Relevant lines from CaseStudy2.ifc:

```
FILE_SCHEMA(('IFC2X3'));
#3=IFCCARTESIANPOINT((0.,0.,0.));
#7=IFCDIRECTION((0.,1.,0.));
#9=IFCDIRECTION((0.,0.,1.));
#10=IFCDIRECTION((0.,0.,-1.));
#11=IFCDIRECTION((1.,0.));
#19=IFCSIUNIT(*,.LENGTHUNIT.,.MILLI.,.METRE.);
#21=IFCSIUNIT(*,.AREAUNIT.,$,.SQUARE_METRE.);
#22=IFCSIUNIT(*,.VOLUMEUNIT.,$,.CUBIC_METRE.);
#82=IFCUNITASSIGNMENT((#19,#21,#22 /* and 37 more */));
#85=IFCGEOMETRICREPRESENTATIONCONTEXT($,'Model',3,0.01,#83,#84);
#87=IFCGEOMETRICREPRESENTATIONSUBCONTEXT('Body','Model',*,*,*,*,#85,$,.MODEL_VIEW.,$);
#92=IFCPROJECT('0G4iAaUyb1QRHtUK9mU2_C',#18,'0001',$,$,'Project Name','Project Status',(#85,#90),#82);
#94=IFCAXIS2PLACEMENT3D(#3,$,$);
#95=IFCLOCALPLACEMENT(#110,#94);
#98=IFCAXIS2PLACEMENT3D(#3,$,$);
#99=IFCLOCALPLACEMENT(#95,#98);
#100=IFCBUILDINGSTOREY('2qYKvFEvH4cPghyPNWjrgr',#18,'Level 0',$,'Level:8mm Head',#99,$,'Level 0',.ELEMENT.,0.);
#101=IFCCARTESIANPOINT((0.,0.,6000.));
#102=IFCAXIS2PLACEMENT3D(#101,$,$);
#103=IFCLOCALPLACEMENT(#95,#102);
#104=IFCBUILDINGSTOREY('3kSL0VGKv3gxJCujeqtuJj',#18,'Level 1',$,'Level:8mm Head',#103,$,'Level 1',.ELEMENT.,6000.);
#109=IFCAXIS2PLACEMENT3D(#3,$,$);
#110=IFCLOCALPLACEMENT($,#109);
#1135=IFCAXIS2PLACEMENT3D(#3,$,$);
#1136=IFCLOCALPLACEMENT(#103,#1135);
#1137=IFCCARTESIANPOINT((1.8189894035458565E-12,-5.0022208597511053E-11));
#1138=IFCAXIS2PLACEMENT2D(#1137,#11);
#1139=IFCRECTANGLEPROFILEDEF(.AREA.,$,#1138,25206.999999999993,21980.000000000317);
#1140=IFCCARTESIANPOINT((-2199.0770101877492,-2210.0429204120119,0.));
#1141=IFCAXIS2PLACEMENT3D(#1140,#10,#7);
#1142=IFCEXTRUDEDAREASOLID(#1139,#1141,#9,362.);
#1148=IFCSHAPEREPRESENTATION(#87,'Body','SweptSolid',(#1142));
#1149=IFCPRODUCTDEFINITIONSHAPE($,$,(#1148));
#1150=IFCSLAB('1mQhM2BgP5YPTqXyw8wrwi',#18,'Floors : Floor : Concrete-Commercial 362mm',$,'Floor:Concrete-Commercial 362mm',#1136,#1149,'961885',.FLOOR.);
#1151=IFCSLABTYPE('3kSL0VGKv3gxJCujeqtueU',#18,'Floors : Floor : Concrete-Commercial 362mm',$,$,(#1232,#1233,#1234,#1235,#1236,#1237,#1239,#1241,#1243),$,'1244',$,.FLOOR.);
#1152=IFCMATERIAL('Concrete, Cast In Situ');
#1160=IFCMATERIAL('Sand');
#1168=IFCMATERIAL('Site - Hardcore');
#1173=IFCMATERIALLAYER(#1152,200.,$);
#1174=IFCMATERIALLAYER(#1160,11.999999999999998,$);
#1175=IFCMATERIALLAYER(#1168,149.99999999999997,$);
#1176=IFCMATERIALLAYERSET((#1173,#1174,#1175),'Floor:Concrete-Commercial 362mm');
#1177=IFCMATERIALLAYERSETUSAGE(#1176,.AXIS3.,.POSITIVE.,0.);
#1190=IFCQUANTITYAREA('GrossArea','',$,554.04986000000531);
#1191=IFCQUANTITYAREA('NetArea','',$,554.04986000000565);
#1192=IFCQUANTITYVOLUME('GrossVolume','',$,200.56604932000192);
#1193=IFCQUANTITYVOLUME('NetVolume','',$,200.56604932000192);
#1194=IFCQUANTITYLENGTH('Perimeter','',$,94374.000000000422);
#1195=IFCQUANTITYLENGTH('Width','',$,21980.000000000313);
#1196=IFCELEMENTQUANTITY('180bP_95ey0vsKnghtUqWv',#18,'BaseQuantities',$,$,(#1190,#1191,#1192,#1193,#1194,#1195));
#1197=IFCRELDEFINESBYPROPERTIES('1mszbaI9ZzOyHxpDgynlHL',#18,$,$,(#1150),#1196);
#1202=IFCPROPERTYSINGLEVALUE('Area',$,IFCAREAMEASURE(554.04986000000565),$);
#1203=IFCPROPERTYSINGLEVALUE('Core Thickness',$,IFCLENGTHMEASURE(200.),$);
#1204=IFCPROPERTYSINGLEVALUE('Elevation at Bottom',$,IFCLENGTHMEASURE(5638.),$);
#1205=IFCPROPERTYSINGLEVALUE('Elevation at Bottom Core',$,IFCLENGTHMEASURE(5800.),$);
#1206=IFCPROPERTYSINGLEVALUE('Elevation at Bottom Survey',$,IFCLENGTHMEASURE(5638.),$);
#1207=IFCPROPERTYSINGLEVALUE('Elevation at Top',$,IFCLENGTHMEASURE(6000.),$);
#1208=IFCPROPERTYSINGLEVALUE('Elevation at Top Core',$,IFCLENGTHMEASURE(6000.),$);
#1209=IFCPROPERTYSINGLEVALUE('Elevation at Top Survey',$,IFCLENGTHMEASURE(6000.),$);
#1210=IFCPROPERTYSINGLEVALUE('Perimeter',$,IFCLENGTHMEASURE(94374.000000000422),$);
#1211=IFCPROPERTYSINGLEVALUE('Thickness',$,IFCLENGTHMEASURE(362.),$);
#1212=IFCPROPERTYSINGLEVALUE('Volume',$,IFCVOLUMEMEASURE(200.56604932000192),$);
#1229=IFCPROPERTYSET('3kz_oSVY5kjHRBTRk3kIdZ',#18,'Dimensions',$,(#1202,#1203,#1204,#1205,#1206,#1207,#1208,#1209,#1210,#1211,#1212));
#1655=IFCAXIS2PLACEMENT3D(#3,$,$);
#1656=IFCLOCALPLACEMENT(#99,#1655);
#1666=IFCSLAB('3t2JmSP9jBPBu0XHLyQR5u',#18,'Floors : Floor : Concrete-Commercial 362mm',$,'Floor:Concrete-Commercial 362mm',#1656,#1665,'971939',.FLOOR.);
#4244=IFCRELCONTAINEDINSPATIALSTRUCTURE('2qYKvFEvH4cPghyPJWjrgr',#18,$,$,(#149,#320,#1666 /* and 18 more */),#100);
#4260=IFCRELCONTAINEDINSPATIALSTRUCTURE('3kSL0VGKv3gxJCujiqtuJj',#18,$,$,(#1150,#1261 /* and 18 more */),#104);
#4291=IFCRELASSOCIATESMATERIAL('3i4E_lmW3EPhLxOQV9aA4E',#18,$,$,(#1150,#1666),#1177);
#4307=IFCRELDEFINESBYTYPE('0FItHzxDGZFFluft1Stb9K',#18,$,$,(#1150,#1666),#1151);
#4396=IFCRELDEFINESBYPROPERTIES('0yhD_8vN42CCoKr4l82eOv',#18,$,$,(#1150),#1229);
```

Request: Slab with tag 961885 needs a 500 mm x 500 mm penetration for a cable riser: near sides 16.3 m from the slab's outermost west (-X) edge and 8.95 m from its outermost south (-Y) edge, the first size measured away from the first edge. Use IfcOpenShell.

```python
import numpy as np
import ifcopenshell
import ifcopenshell.api.feature
import ifcopenshell.api.geometry
import ifcopenshell.api.pset
import ifcopenshell.api.root
import ifcopenshell.geom
import ifcopenshell.util.element
import ifcopenshell.util.placement
import ifcopenshell.util.representation
import ifcopenshell.util.shape
import ifcopenshell.util.unit

model = ifcopenshell.open("CaseStudy2.ifc")
unit_scale = ifcopenshell.util.unit.calculate_unit_scale(model)
area_scale = ifcopenshell.util.unit.calculate_unit_scale(model, "AREAUNIT")
volume_scale = ifcopenshell.util.unit.calculate_unit_scale(model, "VOLUMEUNIT")
settings = ifcopenshell.geom.settings()


def volume(element):
    """Net volume in cubic metres, openings subtracted."""
    shape = ifcopenshell.geom.create_shape(settings, element)
    return ifcopenshell.util.shape.get_volume(shape.geometry)


slab = model.by_guid("1mQhM2BgP5YPTqXyw8wrwi")
before = volume(slab)

# Extent in the slab's own axes, in metres. The edges named are its -X and -Y sides.
slab_shape = ifcopenshell.geom.create_shape(settings, slab)
vertices = ifcopenshell.util.shape.get_vertices(slab_shape.geometry)
x_min, y_min, bottom = vertices.min(axis=0)
top = vertices[:, 2].max()

opening = ifcopenshell.api.root.create_entity(model, ifc_class="IfcOpeningElement", name="Cable riser opening")
context = ifcopenshell.util.representation.get_context(model, "Model", "Body", "MODEL_VIEW")
width, depth = 0.5, 0.5
outline = [(0.0, 0.0), (width, 0.0), (width, depth), (0.0, depth), (0.0, 0.0)]
# Overshoot both faces by 50 mm so the cut is clean.
shape = ifcopenshell.api.geometry.add_slab_representation(
    model, context=context, depth=top - bottom + 0.1, polyline=outline
)
ifcopenshell.api.geometry.assign_representation(model, product=opening, representation=shape)

matrix = ifcopenshell.util.placement.get_local_placement(slab.ObjectPlacement)
matrix[:, 3] = matrix @ np.append(np.array([x_min + 16.3, y_min + 8.95, bottom - 0.05]) / unit_scale, 1.0)
ifcopenshell.api.geometry.edit_object_placement(model, product=opening, matrix=matrix, is_si=False)
ifcopenshell.api.feature.add_feature(model, feature=opening, element=slab)

after = volume(slab)

# Update the slab's stored quantities.
qto = model.by_id(ifcopenshell.util.element.get_pset(slab, "BaseQuantities", should_inherit=False)["id"])
ifcopenshell.api.pset.edit_qto(model, qto=qto, properties={
    "NetArea": after / (top - bottom) / area_scale,
    "NetVolume": after / volume_scale,
})
pset = model.by_id(ifcopenshell.util.element.get_pset(slab, "Dimensions", should_inherit=False)["id"])
ifcopenshell.api.pset.edit_pset(model, pset=pset, properties={
    "Area": model.create_entity("IfcAreaMeasure", after / (top - bottom) / area_scale),
    "Volume": model.create_entity("IfcVolumeMeasure", after / volume_scale),
})

print(f"slab volume {before:.3f} -> {after:.3f} m3")

model.write("CaseStudy2-out.ifc")
```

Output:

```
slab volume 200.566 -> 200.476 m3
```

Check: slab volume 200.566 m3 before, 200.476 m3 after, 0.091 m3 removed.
